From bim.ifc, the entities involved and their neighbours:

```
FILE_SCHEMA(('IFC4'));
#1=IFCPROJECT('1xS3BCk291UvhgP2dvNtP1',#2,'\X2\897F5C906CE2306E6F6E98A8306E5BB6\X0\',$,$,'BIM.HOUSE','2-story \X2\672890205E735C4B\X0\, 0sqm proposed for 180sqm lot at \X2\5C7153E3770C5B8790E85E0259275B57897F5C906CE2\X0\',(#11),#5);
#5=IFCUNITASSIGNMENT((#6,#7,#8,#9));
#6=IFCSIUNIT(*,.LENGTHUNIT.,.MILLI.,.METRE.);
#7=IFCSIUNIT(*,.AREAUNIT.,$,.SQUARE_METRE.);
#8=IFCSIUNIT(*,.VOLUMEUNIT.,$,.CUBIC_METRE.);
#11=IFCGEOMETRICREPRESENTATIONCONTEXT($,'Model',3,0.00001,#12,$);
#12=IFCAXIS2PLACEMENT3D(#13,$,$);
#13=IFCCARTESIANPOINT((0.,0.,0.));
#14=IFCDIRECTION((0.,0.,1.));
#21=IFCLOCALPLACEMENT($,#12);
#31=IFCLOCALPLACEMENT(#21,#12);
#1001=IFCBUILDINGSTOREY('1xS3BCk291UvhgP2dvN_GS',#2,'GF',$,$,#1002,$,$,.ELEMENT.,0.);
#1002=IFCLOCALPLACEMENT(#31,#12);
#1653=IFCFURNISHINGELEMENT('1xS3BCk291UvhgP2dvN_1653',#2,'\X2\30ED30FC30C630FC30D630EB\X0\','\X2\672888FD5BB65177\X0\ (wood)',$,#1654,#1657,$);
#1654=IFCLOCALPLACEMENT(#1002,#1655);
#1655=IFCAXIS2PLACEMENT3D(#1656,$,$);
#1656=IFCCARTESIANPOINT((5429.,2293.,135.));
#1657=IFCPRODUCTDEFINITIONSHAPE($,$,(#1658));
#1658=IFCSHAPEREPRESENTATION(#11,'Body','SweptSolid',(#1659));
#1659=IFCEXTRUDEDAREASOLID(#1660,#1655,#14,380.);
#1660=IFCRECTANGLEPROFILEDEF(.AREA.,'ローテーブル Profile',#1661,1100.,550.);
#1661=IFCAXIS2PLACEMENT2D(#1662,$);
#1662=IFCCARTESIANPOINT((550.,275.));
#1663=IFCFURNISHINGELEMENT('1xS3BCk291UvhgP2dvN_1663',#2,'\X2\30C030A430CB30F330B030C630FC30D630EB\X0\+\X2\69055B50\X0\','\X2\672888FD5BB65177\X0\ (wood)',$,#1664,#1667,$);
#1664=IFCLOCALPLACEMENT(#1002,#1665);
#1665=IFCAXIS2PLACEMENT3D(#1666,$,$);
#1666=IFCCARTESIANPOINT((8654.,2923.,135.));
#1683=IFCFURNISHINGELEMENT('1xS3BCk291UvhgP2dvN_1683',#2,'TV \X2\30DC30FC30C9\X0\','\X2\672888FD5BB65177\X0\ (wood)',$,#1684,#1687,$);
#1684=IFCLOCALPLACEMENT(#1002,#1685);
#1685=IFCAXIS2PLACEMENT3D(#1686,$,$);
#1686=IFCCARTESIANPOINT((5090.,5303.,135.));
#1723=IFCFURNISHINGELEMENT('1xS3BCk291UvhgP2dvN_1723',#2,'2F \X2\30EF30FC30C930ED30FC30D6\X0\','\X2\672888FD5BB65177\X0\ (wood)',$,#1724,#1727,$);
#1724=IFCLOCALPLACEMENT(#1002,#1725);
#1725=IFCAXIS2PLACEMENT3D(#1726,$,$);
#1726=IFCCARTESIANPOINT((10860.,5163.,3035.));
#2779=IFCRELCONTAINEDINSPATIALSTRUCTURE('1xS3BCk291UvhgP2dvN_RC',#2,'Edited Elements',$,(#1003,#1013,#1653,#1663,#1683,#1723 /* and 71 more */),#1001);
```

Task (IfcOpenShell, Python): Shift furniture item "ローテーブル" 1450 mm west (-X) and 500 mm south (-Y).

```python
import ifcopenshell
import ifcopenshell.api.geometry
import ifcopenshell.util.placement

model = ifcopenshell.open("bim.ifc")

item = model.by_id(1653)
matrix = ifcopenshell.util.placement.get_local_placement(item.ObjectPlacement)
matrix[0, 3] -= 1450.0
matrix[1, 3] -= 500.0
ifcopenshell.api.geometry.edit_object_placement(model, product=item, matrix=matrix, is_si=False)

print(ifcopenshell.util.placement.get_local_placement(item.ObjectPlacement).round(3) + 0.0)

model.write("bim_rev.ifc")
```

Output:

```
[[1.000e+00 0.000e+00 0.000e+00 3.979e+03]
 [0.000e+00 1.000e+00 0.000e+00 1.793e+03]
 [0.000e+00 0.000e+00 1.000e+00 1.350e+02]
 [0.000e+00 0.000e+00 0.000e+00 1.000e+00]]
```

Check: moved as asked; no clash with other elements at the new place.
